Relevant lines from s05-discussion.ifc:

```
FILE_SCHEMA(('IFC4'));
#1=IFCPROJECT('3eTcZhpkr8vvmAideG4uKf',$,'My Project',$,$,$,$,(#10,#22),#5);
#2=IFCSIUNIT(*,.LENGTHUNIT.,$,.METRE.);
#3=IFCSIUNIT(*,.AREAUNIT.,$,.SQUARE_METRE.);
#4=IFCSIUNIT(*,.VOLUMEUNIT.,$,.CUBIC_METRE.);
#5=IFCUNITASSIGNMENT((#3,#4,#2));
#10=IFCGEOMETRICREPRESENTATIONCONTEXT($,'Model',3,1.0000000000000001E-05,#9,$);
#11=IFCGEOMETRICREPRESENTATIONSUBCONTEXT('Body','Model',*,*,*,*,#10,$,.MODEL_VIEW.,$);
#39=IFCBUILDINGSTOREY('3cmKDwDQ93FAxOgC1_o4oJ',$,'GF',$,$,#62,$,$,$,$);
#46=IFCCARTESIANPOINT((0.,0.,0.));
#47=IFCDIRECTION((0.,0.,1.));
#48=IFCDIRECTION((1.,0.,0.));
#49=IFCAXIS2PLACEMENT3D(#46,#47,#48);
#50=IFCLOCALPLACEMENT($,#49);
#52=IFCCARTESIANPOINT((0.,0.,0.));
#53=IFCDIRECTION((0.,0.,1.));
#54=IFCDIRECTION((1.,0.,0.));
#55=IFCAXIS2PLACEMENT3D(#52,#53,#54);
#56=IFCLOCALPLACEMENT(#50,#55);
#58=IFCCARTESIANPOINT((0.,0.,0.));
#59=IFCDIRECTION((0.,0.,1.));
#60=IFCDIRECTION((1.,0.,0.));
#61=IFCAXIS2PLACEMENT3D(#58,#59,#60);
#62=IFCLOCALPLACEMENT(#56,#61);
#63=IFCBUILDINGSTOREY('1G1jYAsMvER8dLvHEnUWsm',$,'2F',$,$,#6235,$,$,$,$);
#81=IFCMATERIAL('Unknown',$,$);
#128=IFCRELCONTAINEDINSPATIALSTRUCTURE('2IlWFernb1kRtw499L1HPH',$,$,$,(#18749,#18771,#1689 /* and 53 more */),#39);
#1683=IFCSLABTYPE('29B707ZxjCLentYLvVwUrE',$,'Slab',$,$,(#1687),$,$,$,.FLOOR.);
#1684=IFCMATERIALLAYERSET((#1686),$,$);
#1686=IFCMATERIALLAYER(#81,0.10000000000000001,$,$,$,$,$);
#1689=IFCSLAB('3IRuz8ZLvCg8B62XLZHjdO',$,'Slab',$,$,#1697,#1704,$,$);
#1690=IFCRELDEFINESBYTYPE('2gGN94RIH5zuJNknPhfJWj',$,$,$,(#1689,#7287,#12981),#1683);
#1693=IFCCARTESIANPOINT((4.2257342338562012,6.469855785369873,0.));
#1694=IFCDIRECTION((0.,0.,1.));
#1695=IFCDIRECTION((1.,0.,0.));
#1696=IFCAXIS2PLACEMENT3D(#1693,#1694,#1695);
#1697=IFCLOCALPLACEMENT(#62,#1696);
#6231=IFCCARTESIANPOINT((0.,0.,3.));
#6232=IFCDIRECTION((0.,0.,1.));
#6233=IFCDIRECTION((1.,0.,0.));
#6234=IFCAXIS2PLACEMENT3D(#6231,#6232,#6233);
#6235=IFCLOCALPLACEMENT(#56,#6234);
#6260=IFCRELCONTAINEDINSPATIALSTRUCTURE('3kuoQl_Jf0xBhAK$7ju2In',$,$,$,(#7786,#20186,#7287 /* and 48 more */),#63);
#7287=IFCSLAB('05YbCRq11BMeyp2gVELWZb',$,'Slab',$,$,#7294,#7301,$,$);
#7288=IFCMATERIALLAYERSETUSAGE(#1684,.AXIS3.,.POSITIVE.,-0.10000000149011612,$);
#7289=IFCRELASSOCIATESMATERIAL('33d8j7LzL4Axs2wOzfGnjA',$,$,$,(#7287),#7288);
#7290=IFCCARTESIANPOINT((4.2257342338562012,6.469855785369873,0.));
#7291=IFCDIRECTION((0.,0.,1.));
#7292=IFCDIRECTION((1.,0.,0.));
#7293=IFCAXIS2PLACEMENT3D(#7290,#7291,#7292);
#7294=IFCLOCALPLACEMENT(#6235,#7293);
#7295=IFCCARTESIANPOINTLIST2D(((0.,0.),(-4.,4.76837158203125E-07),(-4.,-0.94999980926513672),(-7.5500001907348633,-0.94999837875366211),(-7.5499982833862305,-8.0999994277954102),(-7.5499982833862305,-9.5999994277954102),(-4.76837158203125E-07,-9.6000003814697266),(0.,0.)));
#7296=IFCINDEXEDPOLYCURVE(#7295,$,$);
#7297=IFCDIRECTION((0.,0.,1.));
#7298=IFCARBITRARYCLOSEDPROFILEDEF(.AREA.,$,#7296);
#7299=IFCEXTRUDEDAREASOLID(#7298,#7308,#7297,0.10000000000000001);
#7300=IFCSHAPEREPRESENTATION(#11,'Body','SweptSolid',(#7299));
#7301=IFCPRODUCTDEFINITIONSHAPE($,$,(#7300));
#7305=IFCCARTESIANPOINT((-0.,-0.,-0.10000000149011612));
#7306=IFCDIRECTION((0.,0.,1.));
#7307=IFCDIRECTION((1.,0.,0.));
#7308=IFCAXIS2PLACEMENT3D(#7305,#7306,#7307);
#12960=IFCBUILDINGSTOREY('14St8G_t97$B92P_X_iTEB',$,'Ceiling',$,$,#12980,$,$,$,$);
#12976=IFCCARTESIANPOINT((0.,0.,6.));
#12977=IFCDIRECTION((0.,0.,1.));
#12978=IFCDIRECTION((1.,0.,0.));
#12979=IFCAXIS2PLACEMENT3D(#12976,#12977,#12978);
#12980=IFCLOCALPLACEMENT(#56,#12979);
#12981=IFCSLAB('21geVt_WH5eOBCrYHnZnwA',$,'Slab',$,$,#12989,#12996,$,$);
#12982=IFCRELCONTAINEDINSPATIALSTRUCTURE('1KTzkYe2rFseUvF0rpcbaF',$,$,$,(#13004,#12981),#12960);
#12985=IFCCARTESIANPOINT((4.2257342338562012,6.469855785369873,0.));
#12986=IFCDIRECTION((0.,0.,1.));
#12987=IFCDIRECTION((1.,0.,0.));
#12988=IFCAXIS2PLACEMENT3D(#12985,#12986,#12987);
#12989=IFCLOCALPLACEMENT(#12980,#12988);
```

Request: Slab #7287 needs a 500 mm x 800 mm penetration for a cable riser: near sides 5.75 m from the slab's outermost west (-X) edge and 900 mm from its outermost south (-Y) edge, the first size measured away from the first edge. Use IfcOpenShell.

```python
import numpy as np
import ifcopenshell
import ifcopenshell.api.feature
import ifcopenshell.api.geometry
import ifcopenshell.api.root
import ifcopenshell.geom
import ifcopenshell.util.placement
import ifcopenshell.util.representation
import ifcopenshell.util.shape
import ifcopenshell.util.unit

model = ifcopenshell.open("s05-discussion.ifc")
unit_scale = ifcopenshell.util.unit.calculate_unit_scale(model)
settings = ifcopenshell.geom.settings()


def volume(element):
    """Net volume in cubic metres, openings subtracted."""
    shape = ifcopenshell.geom.create_shape(settings, element)
    return ifcopenshell.util.shape.get_volume(shape.geometry)


slab = model.by_guid("05YbCRq11BMeyp2gVELWZb")
before = volume(slab)

# Extent in the slab's own axes, in metres. The edges named are its -X and -Y sides.
slab_shape = ifcopenshell.geom.create_shape(settings, slab)
vertices = ifcopenshell.util.shape.get_vertices(slab_shape.geometry)
x_min, y_min, bottom = vertices.min(axis=0)
top = vertices[:, 2].max()

opening = ifcopenshell.api.root.create_entity(model, ifc_class="IfcOpeningElement", name="Cable riser opening", predefined_type="OPENING")
context = ifcopenshell.util.representation.get_context(model, "Model", "Body", "MODEL_VIEW")
width, depth = 0.5, 0.8
outline = [(0.0, 0.0), (width, 0.0), (width, depth), (0.0, depth), (0.0, 0.0)]
# Overshoot both faces by 50 mm so the cut is clean.
shape = ifcopenshell.api.geometry.add_slab_representation(
    model, context=context, depth=top - bottom + 0.1, polyline=outline
)
ifcopenshell.api.geometry.assign_representation(model, product=opening, representation=shape)

matrix = ifcopenshell.util.placement.get_local_placement(slab.ObjectPlacement)
matrix[:, 3] = matrix @ np.append(np.array([x_min + 5.75, y_min + 0.9, bottom - 0.05]) / unit_scale, 1.0)
ifcopenshell.api.geometry.edit_object_placement(model, product=opening, matrix=matrix, is_si=False)
ifcopenshell.api.feature.add_feature(model, feature=opening, element=slab)

after = volume(slab)

print(f"slab volume {before:.3f} -> {after:.3f} m3")

model.write("s05-discussion-out.ifc")
```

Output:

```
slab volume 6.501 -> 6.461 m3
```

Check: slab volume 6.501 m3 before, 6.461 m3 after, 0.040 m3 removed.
